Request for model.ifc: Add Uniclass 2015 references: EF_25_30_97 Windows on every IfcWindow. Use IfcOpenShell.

First a look at what the model holds.

```python
import ifcopenshell

model = ifcopenshell.open("model.ifc")
print(model.schema)
print("classifications:", [c.Name for c in model.by_type("IfcClassification")])
for ifc_class in ("IfcDoor", "IfcRoof", "IfcStair", "IfcWall", "IfcWindow"):
    print(ifc_class, len(model.by_type(ifc_class)))
```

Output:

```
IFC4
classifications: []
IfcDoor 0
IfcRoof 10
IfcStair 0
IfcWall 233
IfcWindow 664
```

```python
import ifcopenshell
import ifcopenshell.api.classification

model = ifcopenshell.open("model.ifc")

system = ifcopenshell.api.classification.add_classification(model, classification="Uniclass 2015")

codes = {
    "IfcWindow": ("EF_25_30_97", "Windows"),
}
for ifc_class, (code, name) in codes.items():
    products = model.by_type(ifc_class)
    ifcopenshell.api.classification.add_reference(
        model, products=products, classification=system, identification=code, name=name
    )
    print(code, len(products))

model.write("model-out.ifc")
```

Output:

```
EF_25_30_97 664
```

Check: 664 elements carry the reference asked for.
